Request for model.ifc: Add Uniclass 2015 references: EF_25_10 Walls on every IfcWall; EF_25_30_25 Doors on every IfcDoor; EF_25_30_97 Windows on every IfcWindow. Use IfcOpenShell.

First a look at what the model holds.

```python
import ifcopenshell

model = ifcopenshell.open("model.ifc")
print(model.schema)
print("classifications:", [c.Name for c in model.by_type("IfcClassification")])
for ifc_class in ("IfcDoor", "IfcRoof", "IfcStair", "IfcWall", "IfcWindow"):
    print(ifc_class, len(model.by_type(ifc_class)))
```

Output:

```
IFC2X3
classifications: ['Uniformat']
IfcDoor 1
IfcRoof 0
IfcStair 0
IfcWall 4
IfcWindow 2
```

```python
import ifcopenshell
import ifcopenshell.api.classification

model = ifcopenshell.open("model.ifc")

# IFC2X3 requires Source and Edition and has no link from the project to the system.
system = model.create_entity("IfcClassification", Source="NBS", Edition="2015", Name="Uniclass 2015")

codes = {
    "IfcWall": ("EF_25_10", "Walls"),
    "IfcDoor": ("EF_25_30_25", "Doors"),
    "IfcWindow": ("EF_25_30_97", "Windows"),
}
for ifc_class, (code, name) in codes.items():
    products = model.by_type(ifc_class)
    ifcopenshell.api.classification.add_reference(
        model, products=products, classification=system, identification=code, name=name
    )
    print(code, len(products))

model.write("model_edited.ifc")
```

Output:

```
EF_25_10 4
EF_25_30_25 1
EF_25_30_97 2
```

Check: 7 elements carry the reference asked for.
